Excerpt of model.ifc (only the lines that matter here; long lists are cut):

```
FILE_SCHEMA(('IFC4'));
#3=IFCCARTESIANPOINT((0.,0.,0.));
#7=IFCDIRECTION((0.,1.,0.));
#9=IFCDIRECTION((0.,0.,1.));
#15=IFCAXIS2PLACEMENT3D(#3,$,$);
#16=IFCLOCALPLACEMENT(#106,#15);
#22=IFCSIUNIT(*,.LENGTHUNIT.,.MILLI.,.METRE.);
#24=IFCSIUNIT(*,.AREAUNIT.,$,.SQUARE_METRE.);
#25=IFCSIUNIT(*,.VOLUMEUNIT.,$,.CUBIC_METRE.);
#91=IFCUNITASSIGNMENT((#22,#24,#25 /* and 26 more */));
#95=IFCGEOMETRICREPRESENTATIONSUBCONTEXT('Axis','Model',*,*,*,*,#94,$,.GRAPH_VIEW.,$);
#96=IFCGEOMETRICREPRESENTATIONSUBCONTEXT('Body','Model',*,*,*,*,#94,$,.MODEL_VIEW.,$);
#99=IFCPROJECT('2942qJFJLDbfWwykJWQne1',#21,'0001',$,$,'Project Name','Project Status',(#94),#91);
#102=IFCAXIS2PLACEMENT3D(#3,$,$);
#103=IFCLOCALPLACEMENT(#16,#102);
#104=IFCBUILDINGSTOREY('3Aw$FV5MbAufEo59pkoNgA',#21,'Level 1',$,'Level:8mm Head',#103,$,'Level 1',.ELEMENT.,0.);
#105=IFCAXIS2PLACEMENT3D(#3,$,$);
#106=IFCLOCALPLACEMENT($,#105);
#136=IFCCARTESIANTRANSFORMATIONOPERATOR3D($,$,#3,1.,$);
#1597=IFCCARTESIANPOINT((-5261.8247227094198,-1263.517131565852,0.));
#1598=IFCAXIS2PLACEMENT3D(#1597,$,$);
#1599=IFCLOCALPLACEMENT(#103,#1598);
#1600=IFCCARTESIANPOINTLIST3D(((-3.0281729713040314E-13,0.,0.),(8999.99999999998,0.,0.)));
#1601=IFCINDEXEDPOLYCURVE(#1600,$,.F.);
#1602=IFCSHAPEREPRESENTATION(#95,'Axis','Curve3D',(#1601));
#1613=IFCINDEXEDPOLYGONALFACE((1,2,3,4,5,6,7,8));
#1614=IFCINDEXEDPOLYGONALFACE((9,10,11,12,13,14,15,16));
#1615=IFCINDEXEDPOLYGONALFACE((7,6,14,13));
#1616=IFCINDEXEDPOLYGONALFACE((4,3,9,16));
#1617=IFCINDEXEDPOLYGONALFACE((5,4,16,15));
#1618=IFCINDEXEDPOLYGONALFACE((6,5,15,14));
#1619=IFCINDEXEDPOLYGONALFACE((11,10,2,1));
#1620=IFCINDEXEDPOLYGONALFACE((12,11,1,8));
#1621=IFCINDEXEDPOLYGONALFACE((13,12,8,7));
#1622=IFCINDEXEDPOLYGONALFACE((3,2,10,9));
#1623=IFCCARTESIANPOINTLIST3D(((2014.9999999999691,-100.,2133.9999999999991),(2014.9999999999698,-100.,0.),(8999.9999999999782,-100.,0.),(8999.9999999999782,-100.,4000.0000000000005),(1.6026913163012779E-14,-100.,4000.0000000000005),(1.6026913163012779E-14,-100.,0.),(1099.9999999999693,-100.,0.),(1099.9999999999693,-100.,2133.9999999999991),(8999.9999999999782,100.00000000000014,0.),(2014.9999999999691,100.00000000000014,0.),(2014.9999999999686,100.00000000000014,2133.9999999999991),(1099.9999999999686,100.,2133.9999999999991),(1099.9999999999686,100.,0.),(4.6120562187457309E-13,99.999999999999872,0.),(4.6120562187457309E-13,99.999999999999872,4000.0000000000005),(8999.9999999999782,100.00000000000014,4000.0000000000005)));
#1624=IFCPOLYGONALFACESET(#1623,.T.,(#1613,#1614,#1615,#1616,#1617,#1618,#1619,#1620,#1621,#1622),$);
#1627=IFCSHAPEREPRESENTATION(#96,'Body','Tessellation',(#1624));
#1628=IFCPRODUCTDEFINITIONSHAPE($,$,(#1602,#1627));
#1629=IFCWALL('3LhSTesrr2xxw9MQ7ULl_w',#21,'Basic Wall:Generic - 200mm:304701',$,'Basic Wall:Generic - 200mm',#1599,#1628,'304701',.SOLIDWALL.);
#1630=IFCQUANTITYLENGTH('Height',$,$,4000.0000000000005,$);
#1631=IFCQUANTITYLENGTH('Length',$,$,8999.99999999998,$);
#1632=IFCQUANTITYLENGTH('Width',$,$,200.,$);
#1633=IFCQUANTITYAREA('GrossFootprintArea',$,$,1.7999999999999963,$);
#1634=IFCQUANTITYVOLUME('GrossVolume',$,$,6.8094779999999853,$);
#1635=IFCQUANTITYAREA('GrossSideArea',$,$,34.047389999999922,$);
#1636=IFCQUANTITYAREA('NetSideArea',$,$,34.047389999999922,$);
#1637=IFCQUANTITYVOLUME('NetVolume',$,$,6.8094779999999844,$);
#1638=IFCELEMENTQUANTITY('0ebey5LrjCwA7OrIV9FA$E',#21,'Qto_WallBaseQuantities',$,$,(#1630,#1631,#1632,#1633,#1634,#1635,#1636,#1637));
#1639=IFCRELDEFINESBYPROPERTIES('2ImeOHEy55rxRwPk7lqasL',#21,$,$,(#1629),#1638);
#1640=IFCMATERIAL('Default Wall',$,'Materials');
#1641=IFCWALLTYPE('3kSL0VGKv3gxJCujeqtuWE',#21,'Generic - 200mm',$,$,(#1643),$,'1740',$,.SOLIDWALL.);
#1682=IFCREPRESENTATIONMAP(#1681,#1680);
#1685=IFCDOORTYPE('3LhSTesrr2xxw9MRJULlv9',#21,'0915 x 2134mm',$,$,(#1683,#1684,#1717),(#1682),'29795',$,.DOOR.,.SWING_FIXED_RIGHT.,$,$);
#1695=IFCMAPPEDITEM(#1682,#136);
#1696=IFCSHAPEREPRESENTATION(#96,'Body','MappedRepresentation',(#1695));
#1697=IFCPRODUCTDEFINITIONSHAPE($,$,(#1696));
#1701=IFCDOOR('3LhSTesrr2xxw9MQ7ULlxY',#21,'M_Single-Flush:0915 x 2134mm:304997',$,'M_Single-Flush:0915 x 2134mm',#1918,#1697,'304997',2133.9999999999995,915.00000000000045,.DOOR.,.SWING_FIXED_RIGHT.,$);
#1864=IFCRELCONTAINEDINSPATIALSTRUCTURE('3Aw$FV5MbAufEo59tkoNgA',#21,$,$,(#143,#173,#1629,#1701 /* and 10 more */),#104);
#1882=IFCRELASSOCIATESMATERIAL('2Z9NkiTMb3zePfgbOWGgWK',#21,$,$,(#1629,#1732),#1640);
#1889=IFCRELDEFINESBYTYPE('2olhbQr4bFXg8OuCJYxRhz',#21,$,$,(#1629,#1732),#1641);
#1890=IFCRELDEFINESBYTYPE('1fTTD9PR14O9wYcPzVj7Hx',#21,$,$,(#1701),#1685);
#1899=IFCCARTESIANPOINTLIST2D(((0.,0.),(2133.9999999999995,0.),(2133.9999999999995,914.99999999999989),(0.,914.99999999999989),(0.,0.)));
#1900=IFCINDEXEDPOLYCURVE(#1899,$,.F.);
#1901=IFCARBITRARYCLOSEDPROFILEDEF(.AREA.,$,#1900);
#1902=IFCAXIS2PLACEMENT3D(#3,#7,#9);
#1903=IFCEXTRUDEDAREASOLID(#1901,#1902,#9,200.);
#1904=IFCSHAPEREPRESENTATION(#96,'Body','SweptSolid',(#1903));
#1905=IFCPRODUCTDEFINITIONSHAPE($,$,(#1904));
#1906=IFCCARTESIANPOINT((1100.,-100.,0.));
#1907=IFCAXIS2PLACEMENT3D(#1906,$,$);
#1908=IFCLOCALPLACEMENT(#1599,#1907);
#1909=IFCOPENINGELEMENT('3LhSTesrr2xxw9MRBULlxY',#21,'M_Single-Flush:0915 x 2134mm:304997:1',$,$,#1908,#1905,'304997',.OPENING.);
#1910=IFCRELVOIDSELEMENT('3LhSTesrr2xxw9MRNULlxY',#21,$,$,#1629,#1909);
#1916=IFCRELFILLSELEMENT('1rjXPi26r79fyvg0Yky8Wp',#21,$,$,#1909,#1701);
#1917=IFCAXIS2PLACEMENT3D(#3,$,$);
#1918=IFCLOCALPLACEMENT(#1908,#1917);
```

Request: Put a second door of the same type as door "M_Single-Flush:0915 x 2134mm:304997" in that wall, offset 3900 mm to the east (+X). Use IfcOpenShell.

```python
import ifcopenshell
import ifcopenshell.api.feature
import ifcopenshell.api.geometry
import ifcopenshell.api.pset
import ifcopenshell.api.root
import ifcopenshell.geom
import ifcopenshell.util.element
import ifcopenshell.util.placement
import ifcopenshell.util.shape
import ifcopenshell.util.unit

model = ifcopenshell.open("model.ifc")
unit_scale = ifcopenshell.util.unit.calculate_unit_scale(model)
area_scale = ifcopenshell.util.unit.calculate_unit_scale(model, "AREAUNIT")
volume_scale = ifcopenshell.util.unit.calculate_unit_scale(model, "VOLUMEUNIT")
settings = ifcopenshell.geom.settings()


def volume(element):
    """Net volume in cubic metres, openings subtracted."""
    shape = ifcopenshell.geom.create_shape(settings, element)
    return ifcopenshell.util.shape.get_volume(shape.geometry)


def reuse_history(source, copy):
    """copy_class also copies each property set's owner history, people and application; keep the originals."""
    for rel in copy.IsDefinedBy:
        if rel.is_a("IfcRelDefinesByProperties") and (history := rel.RelatingPropertyDefinition.OwnerHistory):
            rel.RelatingPropertyDefinition.OwnerHistory = source.OwnerHistory
            ifcopenshell.util.element.remove_deep2(model, history)


door = model.by_id(1701)
opening = door.FillsVoids[0].RelatingOpeningElement
wall = opening.VoidsElements[0].RelatingBuildingElement
before = volume(wall)
shift = ifcopenshell.util.placement.get_local_placement(wall.ObjectPlacement)[:3, 0] * 3.9 / unit_scale

# copy_class copies the void relationship, type, container and properties, but no geometry.
new_opening = ifcopenshell.api.root.copy_class(model, product=opening)
new_opening.Representation = ifcopenshell.util.element.copy_deep(
    model, opening.Representation, exclude=["IfcGeometricRepresentationContext", "IfcRepresentationMap"]
)
new_opening.Name = "M_Single-Flush:0915 x 2134mm"
new_opening.Tag = None
reuse_history(opening, new_opening)
new_door = ifcopenshell.api.root.copy_class(model, product=door)
new_door.Representation = ifcopenshell.util.element.copy_deep(
    model, door.Representation, exclude=["IfcGeometricRepresentationContext", "IfcRepresentationMap"]
)
new_door.Name = "M_Single-Flush:0915 x 2134mm"
new_door.Tag = None
reuse_history(door, new_door)
ifcopenshell.api.feature.add_filling(model, opening=new_opening, element=new_door)

for old, new in ((opening, new_opening), (door, new_door)):
    matrix = ifcopenshell.util.placement.get_local_placement(old.ObjectPlacement)
    matrix[:3, 3] += shift
    ifcopenshell.api.geometry.edit_object_placement(model, product=new, matrix=matrix, is_si=False)

after = volume(wall)
thickness = 0.2  # wall thickness in metres

# Update the wall's stored quantities.
qto = model.by_id(ifcopenshell.util.element.get_pset(wall, "Qto_WallBaseQuantities", should_inherit=False)["id"])
ifcopenshell.api.pset.edit_qto(model, qto=qto, properties={
    "NetSideArea": after / thickness / area_scale,
    "NetVolume": after / volume_scale,
})

print(f"wall volume {before:.3f} -> {after:.3f} m3")

model.write("model-out.ifc")
```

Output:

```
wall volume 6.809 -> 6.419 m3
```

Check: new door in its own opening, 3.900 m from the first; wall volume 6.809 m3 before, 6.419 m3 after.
